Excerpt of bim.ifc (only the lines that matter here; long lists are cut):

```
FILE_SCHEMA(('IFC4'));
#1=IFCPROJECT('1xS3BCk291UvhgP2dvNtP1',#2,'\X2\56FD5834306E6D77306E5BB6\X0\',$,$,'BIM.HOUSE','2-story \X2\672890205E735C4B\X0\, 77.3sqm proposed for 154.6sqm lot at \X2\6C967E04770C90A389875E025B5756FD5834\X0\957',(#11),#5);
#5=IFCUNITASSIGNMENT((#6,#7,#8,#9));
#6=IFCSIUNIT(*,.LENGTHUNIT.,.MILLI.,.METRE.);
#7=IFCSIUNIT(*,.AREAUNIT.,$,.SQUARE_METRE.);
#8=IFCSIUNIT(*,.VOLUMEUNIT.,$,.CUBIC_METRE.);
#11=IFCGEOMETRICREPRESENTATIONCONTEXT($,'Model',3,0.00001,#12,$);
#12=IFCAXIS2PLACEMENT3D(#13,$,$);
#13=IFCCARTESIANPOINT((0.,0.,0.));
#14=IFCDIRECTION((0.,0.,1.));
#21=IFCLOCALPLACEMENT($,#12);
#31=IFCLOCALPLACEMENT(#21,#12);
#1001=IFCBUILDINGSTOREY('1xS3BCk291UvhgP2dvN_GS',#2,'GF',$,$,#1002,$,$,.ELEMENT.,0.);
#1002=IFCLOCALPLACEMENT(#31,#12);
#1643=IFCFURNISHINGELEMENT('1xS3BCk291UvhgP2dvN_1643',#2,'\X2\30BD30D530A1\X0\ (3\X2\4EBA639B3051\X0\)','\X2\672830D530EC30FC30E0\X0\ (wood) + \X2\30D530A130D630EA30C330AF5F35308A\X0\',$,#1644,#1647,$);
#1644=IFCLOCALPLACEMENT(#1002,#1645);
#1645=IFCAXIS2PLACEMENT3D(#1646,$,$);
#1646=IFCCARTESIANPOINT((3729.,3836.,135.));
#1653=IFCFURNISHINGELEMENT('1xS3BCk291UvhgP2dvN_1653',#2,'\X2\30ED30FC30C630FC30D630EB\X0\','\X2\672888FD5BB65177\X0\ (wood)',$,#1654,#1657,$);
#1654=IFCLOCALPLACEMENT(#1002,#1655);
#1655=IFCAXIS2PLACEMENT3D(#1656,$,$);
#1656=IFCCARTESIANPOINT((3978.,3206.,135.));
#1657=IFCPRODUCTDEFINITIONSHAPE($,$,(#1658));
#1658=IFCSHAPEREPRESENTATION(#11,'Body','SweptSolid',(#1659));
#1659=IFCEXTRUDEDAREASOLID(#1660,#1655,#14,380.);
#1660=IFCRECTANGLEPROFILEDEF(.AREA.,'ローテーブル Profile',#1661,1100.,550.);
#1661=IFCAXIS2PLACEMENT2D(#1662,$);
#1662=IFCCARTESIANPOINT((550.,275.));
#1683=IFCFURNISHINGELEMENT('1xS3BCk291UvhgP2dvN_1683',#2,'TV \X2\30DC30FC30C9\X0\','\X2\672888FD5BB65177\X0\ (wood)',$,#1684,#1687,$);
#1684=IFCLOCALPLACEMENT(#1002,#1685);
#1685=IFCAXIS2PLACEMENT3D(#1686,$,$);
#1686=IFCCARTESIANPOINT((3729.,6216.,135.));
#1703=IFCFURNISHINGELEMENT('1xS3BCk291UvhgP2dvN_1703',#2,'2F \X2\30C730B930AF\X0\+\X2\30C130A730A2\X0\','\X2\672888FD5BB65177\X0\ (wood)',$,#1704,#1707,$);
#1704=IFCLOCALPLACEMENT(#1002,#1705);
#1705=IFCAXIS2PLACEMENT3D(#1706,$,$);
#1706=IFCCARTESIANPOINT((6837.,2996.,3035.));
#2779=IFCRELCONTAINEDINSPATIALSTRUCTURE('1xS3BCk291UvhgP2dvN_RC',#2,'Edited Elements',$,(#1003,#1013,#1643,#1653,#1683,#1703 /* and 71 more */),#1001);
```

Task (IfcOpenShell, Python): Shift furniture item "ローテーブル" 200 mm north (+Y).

```python
import ifcopenshell
import ifcopenshell.api.geometry
import ifcopenshell.util.placement

model = ifcopenshell.open("bim.ifc")

item = model.by_guid("1xS3BCk291UvhgP2dvN_1653")
matrix = ifcopenshell.util.placement.get_local_placement(item.ObjectPlacement)
matrix[1, 3] += 200.0
ifcopenshell.api.geometry.edit_object_placement(model, product=item, matrix=matrix, is_si=False)

print(ifcopenshell.util.placement.get_local_placement(item.ObjectPlacement).round(3) + 0.0)

model.write("bim_rev.ifc")
```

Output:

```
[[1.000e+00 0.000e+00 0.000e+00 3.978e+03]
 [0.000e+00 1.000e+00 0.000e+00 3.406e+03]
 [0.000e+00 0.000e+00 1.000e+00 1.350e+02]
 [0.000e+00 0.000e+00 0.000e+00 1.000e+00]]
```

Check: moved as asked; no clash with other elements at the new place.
